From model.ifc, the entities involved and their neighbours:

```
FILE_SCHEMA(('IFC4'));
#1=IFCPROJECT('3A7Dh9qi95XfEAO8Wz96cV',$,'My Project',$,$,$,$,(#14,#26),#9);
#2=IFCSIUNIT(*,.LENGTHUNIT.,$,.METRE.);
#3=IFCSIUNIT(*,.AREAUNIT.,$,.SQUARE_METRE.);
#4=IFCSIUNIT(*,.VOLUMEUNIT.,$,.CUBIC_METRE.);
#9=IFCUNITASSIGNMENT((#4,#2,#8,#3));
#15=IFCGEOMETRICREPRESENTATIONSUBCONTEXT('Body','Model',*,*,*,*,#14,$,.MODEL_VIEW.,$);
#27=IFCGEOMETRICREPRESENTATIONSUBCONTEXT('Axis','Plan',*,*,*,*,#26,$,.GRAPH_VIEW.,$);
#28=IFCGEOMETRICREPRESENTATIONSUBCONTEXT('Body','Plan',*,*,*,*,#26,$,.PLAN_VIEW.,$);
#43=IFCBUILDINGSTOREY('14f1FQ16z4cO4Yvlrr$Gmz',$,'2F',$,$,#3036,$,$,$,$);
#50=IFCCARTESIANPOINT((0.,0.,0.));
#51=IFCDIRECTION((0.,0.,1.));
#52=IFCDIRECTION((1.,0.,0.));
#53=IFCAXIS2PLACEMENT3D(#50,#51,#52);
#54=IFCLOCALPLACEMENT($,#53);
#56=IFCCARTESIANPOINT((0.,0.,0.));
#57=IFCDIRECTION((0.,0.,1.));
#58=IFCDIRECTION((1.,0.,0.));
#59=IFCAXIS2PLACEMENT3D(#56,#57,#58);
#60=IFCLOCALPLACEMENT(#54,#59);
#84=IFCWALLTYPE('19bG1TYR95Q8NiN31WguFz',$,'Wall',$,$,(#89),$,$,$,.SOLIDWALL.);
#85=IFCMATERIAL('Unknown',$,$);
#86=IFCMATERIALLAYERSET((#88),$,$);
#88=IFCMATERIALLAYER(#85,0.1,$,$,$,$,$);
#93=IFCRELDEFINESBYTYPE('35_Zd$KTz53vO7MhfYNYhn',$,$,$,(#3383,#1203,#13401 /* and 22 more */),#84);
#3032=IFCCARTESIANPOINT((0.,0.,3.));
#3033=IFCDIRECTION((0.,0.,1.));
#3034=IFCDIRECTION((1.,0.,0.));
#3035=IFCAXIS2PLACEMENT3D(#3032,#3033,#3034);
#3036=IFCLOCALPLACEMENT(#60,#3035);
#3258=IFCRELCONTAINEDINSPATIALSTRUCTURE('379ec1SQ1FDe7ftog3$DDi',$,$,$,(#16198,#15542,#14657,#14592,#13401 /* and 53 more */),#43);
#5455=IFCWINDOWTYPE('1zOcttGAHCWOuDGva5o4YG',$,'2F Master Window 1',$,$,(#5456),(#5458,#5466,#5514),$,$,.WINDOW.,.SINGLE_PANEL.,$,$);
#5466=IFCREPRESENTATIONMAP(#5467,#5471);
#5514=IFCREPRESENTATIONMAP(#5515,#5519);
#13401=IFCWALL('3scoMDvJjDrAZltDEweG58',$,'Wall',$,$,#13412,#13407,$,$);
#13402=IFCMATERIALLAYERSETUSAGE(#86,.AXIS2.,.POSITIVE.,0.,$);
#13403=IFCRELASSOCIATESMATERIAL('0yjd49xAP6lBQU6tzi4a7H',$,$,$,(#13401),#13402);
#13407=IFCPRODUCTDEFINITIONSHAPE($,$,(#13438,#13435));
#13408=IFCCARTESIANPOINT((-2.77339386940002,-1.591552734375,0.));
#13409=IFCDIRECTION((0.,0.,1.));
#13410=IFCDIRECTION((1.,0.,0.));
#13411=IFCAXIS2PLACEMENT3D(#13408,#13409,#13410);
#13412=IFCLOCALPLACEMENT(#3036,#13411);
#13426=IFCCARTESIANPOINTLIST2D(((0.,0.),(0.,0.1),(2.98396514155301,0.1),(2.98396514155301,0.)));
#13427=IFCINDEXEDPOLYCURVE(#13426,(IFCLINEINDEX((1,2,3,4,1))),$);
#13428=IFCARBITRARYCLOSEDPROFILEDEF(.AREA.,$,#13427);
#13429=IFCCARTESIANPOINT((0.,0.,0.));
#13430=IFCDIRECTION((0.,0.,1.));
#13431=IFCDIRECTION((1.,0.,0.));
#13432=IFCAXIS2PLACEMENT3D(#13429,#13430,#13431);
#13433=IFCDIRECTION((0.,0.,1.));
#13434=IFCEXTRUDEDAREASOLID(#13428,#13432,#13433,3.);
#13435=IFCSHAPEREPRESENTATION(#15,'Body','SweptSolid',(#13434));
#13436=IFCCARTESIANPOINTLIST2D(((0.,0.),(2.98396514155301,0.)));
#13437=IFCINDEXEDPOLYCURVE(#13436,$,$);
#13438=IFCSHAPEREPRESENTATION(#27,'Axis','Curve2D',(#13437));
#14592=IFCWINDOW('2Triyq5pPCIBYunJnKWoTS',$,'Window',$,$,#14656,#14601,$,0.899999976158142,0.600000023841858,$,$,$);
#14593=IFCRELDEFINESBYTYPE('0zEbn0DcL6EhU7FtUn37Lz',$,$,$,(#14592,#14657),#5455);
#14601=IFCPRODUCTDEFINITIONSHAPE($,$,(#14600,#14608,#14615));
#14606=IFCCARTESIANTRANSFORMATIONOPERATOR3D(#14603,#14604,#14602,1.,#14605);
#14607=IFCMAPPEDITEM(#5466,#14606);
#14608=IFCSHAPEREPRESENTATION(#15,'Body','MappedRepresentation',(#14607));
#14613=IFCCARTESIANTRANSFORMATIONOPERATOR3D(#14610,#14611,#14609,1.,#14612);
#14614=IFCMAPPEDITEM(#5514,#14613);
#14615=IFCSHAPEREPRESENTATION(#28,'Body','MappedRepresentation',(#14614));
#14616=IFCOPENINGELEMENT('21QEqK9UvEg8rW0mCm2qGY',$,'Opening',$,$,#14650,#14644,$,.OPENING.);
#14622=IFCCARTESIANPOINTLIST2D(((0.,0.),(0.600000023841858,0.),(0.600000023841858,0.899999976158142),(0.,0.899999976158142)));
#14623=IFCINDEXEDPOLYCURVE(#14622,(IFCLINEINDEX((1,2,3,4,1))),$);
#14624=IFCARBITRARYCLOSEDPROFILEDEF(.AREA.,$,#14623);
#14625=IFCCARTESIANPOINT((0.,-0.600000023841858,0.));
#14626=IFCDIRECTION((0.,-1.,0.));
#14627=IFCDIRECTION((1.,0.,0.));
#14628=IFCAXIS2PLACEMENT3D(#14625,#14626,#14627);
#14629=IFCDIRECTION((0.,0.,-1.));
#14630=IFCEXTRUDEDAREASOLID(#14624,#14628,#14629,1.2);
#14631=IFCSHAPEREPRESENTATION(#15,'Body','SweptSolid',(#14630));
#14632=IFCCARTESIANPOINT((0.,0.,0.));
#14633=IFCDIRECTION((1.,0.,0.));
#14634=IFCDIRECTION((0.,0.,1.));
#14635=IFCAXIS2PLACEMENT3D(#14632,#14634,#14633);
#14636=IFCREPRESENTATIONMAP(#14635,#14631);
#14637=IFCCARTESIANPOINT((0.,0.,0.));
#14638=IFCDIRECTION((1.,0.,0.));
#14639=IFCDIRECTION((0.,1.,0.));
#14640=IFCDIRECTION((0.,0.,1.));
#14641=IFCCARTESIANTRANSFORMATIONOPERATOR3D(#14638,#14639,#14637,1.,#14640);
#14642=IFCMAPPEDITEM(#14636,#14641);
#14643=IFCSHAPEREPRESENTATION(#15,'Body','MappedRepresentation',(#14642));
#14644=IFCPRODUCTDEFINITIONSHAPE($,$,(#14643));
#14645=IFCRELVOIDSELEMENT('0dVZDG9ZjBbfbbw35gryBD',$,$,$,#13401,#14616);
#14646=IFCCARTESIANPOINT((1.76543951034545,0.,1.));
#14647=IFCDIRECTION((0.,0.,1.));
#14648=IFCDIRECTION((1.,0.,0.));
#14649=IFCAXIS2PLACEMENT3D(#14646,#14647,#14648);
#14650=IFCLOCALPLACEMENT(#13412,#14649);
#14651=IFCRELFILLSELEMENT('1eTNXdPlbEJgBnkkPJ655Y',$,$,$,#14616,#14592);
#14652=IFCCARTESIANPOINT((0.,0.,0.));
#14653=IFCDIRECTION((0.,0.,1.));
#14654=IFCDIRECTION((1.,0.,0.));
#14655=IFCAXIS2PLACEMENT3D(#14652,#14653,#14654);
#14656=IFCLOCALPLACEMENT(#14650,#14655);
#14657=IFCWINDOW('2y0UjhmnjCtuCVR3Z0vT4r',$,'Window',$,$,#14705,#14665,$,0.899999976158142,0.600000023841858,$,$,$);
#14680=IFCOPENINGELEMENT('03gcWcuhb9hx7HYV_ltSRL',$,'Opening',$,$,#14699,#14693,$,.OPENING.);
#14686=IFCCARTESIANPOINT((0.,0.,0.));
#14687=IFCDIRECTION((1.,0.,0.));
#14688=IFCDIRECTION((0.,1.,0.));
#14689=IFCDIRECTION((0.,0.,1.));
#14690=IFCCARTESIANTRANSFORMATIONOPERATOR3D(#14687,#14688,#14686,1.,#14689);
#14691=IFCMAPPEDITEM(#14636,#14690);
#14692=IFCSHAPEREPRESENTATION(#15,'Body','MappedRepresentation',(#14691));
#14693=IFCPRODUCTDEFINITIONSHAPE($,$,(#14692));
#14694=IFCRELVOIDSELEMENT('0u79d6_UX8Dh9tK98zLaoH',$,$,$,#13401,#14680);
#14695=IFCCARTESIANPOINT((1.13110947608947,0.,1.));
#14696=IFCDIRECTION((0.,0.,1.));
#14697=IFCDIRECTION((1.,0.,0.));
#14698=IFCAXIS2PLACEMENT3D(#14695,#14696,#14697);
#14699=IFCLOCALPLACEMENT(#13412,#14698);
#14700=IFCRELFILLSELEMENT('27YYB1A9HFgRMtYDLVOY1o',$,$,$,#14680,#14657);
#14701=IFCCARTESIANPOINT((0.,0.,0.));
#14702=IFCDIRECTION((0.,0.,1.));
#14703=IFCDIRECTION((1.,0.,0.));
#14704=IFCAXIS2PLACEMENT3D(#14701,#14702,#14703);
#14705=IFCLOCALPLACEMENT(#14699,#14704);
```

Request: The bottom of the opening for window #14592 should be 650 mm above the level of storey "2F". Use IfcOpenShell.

```python
import numpy as np
import ifcopenshell
import ifcopenshell.api.geometry
import ifcopenshell.geom
import ifcopenshell.util.element
import ifcopenshell.util.placement
import ifcopenshell.util.shape
import ifcopenshell.util.unit

model = ifcopenshell.open("model.ifc")
unit_scale = ifcopenshell.util.unit.calculate_unit_scale(model)

window = model.by_guid("2Triyq5pPCIBYunJnKWoTS")
opening = window.FillsVoids[0].RelatingOpeningElement
storey = ifcopenshell.util.element.get_container(window, ifc_class="IfcBuildingStorey")
level = ifcopenshell.util.placement.get_local_placement(storey.ObjectPlacement)[2, 3]

# The opening's origin need not be at the sill, so measure its lowest point.
shape = ifcopenshell.geom.create_shape(ifcopenshell.geom.settings(), opening)
bottom = ifcopenshell.util.shape.get_shape_bottom_elevation(shape, shape.geometry) / unit_scale
dz = level + 0.65 - bottom

shift = np.array([0.0, 0.0, dz])
# The window is placed relative to its opening, so it follows when the opening moves.
matrix = ifcopenshell.util.placement.get_local_placement(opening.ObjectPlacement)
matrix[:3, 3] += shift
ifcopenshell.api.geometry.edit_object_placement(
    model, product=opening, matrix=matrix, is_si=False, should_transform_children=True
)

print(f"moved by {dz * unit_scale:+.3f} m")

model.write("model_updated.ifc")
```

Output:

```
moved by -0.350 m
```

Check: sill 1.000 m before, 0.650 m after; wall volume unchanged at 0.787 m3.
